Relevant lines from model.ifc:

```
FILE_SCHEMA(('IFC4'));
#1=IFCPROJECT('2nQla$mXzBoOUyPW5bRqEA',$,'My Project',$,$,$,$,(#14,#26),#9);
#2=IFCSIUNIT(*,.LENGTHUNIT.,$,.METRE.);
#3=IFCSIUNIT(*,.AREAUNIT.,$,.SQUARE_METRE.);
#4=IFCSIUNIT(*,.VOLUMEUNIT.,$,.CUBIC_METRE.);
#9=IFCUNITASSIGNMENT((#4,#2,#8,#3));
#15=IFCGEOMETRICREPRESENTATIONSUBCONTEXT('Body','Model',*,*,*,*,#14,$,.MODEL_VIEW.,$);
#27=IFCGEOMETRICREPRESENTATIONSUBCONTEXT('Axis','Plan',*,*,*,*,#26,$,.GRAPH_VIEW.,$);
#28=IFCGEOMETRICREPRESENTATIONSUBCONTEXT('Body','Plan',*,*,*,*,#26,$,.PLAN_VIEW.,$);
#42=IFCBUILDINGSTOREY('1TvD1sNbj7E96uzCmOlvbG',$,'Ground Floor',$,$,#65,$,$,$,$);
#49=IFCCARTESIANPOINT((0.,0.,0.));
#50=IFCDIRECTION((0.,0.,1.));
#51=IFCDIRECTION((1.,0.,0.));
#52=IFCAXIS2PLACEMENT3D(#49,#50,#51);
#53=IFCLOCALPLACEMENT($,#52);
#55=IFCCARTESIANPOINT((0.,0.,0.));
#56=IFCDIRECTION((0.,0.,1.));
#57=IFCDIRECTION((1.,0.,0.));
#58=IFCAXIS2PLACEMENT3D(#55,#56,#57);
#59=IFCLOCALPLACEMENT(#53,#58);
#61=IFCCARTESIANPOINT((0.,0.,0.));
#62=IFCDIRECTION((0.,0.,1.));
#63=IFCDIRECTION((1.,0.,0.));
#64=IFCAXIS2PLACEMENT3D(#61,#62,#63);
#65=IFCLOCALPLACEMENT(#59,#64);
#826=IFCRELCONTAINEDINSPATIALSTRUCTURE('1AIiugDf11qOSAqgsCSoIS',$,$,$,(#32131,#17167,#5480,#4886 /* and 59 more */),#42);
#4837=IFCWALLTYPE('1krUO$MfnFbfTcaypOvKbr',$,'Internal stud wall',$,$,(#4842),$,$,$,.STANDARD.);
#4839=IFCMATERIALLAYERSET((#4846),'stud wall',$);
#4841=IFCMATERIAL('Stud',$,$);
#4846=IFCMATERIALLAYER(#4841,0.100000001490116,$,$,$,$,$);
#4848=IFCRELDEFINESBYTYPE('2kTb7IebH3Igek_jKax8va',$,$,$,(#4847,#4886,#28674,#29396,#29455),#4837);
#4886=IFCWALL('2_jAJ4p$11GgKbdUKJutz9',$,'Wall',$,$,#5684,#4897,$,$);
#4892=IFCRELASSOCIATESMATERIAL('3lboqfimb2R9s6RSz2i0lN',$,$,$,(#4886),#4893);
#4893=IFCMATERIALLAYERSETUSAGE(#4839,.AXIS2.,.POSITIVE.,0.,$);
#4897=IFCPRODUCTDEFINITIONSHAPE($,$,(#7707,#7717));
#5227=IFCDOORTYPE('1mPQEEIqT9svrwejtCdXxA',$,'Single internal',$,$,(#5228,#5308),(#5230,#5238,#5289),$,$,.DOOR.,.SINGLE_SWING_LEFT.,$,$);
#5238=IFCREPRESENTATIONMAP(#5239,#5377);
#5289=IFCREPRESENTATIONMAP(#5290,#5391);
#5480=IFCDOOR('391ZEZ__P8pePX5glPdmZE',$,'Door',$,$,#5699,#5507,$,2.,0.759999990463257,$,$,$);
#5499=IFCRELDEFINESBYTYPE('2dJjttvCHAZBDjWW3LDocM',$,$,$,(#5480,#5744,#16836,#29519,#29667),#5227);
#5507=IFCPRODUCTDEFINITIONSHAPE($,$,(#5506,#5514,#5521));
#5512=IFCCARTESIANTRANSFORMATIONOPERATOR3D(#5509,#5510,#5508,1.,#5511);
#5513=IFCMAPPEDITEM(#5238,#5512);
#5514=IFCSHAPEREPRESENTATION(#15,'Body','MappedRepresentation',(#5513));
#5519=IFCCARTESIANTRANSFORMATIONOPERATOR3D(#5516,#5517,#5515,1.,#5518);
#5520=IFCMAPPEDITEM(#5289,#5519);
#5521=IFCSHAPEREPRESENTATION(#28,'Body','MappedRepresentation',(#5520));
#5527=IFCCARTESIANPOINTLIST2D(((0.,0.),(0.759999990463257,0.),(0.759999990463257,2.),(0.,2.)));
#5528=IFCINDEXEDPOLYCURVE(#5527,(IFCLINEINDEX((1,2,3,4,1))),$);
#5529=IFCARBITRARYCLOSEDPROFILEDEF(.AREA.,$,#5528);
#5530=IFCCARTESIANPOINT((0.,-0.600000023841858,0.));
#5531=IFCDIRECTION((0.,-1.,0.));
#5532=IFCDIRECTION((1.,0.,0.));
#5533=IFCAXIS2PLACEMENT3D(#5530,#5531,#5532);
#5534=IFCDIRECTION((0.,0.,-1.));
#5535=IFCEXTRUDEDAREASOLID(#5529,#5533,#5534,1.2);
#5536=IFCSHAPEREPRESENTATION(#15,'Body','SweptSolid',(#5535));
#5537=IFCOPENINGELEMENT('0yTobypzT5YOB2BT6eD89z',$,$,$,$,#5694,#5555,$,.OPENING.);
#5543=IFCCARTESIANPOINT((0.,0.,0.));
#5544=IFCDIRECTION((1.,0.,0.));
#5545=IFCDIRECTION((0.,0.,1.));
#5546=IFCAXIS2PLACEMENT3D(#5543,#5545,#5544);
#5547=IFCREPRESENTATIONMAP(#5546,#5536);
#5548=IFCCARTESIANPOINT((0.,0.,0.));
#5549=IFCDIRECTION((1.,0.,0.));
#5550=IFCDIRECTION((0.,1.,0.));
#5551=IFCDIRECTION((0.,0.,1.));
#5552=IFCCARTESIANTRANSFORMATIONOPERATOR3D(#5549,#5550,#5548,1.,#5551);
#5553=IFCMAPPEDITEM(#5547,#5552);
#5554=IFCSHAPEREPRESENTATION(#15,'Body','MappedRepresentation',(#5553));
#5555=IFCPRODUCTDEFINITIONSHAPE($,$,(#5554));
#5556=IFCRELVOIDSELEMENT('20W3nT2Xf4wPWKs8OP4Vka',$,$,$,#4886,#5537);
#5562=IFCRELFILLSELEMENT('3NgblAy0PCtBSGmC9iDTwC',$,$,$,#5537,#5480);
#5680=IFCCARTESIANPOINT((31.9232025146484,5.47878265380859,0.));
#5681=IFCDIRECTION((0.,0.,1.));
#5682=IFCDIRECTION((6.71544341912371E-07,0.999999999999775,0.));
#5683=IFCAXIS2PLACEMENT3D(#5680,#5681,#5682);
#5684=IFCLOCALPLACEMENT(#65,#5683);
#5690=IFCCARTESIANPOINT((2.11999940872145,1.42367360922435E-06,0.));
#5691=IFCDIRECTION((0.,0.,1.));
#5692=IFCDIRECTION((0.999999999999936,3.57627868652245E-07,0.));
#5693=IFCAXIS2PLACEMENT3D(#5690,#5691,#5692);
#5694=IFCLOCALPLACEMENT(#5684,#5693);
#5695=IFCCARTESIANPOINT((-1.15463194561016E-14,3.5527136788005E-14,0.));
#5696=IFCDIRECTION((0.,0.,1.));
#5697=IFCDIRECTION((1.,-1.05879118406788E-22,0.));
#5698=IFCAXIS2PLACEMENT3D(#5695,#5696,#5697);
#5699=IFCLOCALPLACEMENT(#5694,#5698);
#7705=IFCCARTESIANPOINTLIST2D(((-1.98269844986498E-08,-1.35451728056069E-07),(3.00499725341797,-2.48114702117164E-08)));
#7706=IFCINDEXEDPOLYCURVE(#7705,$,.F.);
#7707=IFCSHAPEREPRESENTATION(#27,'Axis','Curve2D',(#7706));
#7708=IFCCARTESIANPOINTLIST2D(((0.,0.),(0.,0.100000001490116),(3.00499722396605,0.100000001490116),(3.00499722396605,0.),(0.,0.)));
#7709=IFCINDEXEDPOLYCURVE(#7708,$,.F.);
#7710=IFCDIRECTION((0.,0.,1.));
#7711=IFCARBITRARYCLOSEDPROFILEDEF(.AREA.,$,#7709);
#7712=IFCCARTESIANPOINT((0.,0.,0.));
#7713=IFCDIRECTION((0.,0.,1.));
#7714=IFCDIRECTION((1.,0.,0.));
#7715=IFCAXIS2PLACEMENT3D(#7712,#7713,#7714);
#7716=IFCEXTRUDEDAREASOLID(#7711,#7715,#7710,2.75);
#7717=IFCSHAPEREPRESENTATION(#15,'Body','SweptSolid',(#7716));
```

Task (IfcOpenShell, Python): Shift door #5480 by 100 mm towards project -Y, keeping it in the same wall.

```python
import ifcopenshell
import ifcopenshell.api.geometry
import ifcopenshell.util.placement

model = ifcopenshell.open("model.ifc")

door = model.by_id(5480)
opening = door.FillsVoids[0].RelatingOpeningElement
wall = opening.VoidsElements[0].RelatingBuildingElement

wall_matrix = ifcopenshell.util.placement.get_local_placement(wall.ObjectPlacement)
shift = wall_matrix[:3, 0] * -0.1
before = ifcopenshell.util.placement.get_local_placement(door.ObjectPlacement)[:3, 3].copy()

# The door is placed relative to its opening, so it follows when the opening moves.
matrix = ifcopenshell.util.placement.get_local_placement(opening.ObjectPlacement)
matrix[:3, 3] += shift
ifcopenshell.api.geometry.edit_object_placement(
    model, product=opening, matrix=matrix, is_si=False, should_transform_children=True
)

after = ifcopenshell.util.placement.get_local_placement(door.ObjectPlacement)[:3, 3]
print("door moved by", (after - before).round(3) + 0.0)

model.write("model_rev.ifc")
```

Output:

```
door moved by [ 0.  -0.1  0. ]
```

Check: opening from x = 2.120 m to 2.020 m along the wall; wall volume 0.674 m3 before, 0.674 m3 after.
